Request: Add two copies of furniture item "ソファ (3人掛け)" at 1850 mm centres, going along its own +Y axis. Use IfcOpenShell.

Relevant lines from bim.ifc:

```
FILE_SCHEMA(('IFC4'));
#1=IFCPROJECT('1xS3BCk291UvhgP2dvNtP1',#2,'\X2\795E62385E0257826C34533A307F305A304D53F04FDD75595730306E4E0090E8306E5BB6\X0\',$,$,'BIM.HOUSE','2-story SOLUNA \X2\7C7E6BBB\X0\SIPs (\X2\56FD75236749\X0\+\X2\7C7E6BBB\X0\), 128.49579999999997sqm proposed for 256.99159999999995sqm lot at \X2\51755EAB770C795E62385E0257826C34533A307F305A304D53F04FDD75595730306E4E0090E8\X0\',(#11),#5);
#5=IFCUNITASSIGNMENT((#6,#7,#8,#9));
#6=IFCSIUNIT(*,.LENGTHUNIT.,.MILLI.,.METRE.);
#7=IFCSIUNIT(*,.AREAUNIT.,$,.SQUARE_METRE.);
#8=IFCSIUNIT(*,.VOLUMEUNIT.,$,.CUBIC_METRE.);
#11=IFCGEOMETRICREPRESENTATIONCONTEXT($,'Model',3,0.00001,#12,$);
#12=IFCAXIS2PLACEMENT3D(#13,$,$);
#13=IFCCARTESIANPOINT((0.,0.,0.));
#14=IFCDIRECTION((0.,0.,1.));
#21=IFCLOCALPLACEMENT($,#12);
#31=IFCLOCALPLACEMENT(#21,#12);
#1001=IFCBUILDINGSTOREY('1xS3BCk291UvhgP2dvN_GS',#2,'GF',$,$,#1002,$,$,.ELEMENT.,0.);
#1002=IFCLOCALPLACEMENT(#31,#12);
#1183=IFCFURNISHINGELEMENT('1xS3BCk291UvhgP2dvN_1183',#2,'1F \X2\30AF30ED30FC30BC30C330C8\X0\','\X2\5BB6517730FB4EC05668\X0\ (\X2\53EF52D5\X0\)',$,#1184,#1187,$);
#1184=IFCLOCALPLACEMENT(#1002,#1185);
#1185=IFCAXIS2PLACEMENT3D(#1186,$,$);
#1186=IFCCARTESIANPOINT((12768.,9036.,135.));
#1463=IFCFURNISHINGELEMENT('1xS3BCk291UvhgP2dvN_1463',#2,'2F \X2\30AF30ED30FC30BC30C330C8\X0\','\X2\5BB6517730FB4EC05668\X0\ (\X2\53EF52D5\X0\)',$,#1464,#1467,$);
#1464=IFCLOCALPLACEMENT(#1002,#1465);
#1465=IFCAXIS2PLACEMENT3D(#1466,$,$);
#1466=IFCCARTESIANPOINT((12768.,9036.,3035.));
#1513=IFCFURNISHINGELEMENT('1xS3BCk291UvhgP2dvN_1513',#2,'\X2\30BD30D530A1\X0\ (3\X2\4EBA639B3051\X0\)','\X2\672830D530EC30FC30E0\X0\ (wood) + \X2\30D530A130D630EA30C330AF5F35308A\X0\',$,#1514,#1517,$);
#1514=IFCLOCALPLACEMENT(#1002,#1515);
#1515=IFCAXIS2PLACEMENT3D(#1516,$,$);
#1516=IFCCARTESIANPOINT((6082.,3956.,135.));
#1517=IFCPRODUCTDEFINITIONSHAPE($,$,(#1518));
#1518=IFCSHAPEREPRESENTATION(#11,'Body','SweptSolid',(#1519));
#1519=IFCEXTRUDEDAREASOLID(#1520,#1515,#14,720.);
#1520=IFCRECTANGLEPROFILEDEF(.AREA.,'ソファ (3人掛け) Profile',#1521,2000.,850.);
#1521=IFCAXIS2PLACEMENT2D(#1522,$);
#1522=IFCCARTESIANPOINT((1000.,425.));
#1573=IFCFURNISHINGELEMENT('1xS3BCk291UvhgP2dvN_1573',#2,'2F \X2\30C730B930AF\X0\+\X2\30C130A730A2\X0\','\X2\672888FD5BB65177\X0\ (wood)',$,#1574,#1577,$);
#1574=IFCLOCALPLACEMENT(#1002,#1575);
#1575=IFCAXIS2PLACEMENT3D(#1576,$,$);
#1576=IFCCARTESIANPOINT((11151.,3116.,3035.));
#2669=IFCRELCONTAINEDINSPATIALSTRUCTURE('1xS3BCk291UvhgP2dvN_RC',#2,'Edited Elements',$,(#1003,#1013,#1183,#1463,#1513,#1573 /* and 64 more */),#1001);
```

```python
import ifcopenshell
import ifcopenshell.api.geometry
import ifcopenshell.api.root
import ifcopenshell.util.element
import ifcopenshell.util.placement
import ifcopenshell.util.unit

model = ifcopenshell.open("bim.ifc")
unit_scale = ifcopenshell.util.unit.calculate_unit_scale(model)


def reuse_history(source, copy):
    """copy_class also copies each property set's owner history, people and application; keep the originals."""
    for rel in copy.IsDefinedBy:
        if rel.is_a("IfcRelDefinesByProperties") and (history := rel.RelatingPropertyDefinition.OwnerHistory):
            rel.RelatingPropertyDefinition.OwnerHistory = source.OwnerHistory
            ifcopenshell.util.element.remove_deep2(model, history)


source = model.by_id(1513)
base = ifcopenshell.util.placement.get_local_placement(source.ObjectPlacement)
step = base[:3, 1] * 1.85 / unit_scale

for i in range(1, 3):
    copy = ifcopenshell.api.root.copy_class(model, product=source)
    copy.Representation = ifcopenshell.util.element.copy_deep(
        model, source.Representation, exclude=["IfcGeometricRepresentationContext", "IfcRepresentationMap"]
    )
    reuse_history(source, copy)
    matrix = base.copy()
    matrix[:3, 3] += i * step
    print("added at", matrix[:3, 3].round(3) + 0.0)
    ifcopenshell.api.geometry.edit_object_placement(model, product=copy, matrix=matrix, is_si=False)

model.write("bim_rev.ifc")
```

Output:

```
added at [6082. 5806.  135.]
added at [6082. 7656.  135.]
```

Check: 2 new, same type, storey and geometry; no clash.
